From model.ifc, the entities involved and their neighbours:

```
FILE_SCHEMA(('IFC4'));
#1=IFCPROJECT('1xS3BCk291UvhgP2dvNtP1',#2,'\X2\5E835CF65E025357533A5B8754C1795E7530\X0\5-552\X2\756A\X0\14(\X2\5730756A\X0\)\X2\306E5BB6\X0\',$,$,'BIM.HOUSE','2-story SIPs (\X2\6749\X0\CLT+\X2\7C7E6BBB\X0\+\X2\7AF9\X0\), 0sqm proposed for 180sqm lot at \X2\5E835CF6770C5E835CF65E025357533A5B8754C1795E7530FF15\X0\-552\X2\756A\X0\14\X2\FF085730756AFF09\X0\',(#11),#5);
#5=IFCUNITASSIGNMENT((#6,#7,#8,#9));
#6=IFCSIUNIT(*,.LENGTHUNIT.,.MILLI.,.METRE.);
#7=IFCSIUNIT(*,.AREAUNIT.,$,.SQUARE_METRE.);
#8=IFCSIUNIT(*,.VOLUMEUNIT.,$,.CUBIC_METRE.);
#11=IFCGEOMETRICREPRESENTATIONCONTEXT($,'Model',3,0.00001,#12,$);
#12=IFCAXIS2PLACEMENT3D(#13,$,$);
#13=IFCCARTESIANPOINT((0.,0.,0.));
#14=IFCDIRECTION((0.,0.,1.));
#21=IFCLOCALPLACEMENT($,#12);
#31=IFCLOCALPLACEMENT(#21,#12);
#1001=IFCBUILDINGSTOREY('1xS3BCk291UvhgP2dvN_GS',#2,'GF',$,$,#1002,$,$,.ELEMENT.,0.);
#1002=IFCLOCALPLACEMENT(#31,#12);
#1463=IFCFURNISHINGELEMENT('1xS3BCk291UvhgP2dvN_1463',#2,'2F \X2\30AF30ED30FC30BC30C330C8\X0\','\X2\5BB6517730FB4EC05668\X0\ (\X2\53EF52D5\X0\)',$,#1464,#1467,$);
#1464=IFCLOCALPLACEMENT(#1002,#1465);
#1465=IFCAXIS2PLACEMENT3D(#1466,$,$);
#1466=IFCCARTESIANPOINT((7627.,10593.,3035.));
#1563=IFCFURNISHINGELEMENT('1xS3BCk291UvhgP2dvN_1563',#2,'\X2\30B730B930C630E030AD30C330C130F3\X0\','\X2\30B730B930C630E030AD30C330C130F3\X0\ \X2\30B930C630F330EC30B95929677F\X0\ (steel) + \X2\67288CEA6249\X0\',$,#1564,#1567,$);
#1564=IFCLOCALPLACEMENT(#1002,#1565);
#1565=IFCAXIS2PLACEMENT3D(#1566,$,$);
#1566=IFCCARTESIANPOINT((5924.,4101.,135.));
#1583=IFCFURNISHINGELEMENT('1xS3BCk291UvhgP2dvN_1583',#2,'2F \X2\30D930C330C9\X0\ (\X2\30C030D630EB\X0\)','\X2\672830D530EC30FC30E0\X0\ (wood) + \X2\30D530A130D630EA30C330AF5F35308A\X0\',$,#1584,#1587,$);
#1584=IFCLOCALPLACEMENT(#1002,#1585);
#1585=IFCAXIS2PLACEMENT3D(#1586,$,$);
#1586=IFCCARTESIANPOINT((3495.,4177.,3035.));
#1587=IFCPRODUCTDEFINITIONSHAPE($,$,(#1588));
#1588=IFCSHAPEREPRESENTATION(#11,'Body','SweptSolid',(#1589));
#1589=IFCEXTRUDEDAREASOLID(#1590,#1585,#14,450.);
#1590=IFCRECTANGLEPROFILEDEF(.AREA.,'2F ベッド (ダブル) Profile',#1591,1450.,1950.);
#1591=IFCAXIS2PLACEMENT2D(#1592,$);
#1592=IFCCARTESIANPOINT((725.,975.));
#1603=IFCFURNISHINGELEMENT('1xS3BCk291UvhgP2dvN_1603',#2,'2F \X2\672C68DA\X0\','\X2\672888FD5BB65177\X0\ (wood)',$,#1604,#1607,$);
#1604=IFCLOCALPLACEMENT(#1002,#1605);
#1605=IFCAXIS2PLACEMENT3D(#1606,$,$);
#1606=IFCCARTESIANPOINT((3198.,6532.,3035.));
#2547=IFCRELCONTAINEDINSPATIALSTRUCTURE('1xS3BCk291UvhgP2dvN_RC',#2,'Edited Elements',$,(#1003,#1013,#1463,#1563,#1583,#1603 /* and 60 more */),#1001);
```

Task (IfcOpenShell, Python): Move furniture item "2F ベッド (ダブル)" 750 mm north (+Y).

```python
import ifcopenshell
import ifcopenshell.api.geometry
import ifcopenshell.util.placement

model = ifcopenshell.open("model.ifc")

item = model.by_guid("1xS3BCk291UvhgP2dvN_1583")
matrix = ifcopenshell.util.placement.get_local_placement(item.ObjectPlacement)
matrix[1, 3] += 750.0
ifcopenshell.api.geometry.edit_object_placement(model, product=item, matrix=matrix, is_si=False)

print(ifcopenshell.util.placement.get_local_placement(item.ObjectPlacement).round(3) + 0.0)

model.write("model_rev.ifc")
```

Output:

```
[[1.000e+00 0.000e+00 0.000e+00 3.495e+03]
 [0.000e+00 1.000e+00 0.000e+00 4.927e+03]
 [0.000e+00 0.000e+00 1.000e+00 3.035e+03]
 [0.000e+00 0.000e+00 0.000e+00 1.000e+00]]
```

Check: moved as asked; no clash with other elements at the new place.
